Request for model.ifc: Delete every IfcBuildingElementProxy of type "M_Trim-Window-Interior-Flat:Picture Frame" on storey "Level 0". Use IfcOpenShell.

First a look at what the model holds.

```python
import ifcopenshell
import ifcopenshell.util.element

model = ifcopenshell.open("model.ifc")
print(model.schema)
storey = next(s for s in model.by_type("IfcBuildingStorey") if s.Name == "Level 0")
proxies = [e for e in ifcopenshell.util.element.get_decomposition(storey) if e.is_a("IfcBuildingElementProxy")]
seen = {}
for e in proxies:
    element_type = ifcopenshell.util.element.get_type(e)
    name = element_type.Name if element_type not in (None, e) else None
    seen[name] = seen.get(name, 0) + 1
for name, count in sorted(seen.items(), key=str):
    print(count, "x", name)
```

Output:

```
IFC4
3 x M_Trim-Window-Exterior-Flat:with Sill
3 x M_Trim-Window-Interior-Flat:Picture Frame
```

```python
import ifcopenshell
import ifcopenshell.api.root
import ifcopenshell.util.element

model = ifcopenshell.open("model.ifc")

storey = next(s for s in model.by_type("IfcBuildingStorey") if s.Name == "Level 0")
proxies = [e for e in ifcopenshell.util.element.get_decomposition(storey) if e.is_a("IfcBuildingElementProxy")]
targets = [e for e in proxies if (t := ifcopenshell.util.element.get_type(e)) not in (None, e) and t.Name == "M_Trim-Window-Interior-Flat:Picture Frame"]

for e in targets:
    ifcopenshell.api.root.remove_product(model, product=e)
print(len(targets), "removed")

model.write("model-out.ifc")
```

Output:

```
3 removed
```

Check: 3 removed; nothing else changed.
